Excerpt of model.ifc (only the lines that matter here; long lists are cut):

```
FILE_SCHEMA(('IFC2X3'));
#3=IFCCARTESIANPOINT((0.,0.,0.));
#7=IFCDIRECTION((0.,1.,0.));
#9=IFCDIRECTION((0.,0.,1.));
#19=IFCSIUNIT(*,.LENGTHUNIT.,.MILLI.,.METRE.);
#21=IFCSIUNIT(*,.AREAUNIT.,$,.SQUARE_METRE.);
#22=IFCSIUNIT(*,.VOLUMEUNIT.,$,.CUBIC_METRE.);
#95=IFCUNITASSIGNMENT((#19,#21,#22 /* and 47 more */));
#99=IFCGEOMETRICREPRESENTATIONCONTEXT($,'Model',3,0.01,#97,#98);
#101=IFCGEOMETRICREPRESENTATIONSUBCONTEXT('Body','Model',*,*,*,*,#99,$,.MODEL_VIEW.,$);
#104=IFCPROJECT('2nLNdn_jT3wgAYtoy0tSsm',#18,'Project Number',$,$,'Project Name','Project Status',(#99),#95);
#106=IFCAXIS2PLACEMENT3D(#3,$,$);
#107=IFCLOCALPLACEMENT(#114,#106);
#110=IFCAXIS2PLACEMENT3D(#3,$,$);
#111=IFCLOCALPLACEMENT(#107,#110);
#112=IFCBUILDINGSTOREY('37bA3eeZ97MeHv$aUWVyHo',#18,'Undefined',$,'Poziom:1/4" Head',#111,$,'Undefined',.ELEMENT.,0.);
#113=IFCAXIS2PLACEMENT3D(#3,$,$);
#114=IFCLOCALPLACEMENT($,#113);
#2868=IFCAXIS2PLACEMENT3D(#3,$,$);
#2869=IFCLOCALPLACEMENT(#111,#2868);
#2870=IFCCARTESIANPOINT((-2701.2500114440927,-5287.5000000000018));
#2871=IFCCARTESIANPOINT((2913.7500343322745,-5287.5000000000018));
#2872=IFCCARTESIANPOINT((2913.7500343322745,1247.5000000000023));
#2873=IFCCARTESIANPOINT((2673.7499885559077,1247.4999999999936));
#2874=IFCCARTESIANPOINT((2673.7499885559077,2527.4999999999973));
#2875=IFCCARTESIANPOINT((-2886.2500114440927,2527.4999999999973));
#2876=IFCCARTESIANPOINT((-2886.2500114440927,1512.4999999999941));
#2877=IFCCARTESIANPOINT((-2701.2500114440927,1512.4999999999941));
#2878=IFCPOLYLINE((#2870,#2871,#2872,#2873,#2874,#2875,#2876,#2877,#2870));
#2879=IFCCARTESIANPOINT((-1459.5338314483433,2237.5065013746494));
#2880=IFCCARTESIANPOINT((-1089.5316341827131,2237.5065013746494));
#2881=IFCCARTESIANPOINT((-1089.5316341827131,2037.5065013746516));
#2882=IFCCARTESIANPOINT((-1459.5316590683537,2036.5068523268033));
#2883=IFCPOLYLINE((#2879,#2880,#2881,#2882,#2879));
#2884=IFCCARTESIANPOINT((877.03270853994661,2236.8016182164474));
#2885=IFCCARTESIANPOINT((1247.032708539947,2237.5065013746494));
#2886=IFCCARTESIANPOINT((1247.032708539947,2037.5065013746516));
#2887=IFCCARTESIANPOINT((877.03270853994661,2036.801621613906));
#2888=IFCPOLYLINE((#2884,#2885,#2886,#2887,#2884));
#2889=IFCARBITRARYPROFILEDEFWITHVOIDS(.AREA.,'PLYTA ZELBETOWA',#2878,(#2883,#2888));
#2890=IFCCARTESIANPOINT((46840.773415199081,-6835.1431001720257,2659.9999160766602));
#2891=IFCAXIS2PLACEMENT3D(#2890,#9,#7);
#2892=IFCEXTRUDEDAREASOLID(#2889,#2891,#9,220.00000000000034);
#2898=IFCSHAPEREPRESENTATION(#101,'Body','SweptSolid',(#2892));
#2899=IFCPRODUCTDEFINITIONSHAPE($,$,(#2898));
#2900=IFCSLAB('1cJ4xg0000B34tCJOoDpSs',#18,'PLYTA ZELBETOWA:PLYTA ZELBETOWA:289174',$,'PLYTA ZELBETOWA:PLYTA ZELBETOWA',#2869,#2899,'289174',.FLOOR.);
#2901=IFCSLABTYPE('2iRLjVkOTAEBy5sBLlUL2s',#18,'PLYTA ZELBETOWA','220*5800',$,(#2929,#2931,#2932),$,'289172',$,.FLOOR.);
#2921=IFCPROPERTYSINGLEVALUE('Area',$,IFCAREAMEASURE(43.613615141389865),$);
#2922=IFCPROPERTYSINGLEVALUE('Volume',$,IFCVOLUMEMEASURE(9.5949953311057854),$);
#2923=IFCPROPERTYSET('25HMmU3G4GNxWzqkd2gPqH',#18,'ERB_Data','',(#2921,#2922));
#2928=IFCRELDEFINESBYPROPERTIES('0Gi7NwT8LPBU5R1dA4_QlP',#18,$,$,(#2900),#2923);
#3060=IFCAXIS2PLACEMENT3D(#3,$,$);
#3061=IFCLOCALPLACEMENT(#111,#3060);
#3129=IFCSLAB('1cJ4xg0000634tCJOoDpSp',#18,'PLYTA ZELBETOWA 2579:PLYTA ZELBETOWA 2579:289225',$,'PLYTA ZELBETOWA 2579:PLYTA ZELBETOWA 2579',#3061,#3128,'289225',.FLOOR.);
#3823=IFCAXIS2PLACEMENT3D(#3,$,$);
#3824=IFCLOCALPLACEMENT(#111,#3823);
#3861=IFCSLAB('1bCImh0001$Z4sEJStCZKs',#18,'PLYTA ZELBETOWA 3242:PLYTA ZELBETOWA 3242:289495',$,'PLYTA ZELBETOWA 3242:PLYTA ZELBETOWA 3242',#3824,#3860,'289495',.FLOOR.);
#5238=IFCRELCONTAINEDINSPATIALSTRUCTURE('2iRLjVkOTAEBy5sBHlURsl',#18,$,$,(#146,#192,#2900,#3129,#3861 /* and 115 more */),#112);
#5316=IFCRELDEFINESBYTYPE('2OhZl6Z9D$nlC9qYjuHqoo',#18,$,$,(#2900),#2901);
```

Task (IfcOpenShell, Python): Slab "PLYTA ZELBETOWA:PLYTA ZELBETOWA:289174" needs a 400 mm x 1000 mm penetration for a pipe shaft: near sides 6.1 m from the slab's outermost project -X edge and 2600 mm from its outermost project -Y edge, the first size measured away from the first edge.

```python
import numpy as np
import ifcopenshell
import ifcopenshell.api.feature
import ifcopenshell.api.geometry
import ifcopenshell.api.pset
import ifcopenshell.api.root
import ifcopenshell.geom
import ifcopenshell.util.element
import ifcopenshell.util.placement
import ifcopenshell.util.representation
import ifcopenshell.util.shape
import ifcopenshell.util.unit

model = ifcopenshell.open("model.ifc")
unit_scale = ifcopenshell.util.unit.calculate_unit_scale(model)
area_scale = ifcopenshell.util.unit.calculate_unit_scale(model, "AREAUNIT")
volume_scale = ifcopenshell.util.unit.calculate_unit_scale(model, "VOLUMEUNIT")
settings = ifcopenshell.geom.settings()


def volume(element):
    """Net volume in cubic metres, openings subtracted."""
    shape = ifcopenshell.geom.create_shape(settings, element)
    return ifcopenshell.util.shape.get_volume(shape.geometry)


slab = model.by_guid("1cJ4xg0000B34tCJOoDpSs")
before = volume(slab)

# Extent in the slab's own axes, in metres. The edges named are its -X and -Y sides.
slab_shape = ifcopenshell.geom.create_shape(settings, slab)
vertices = ifcopenshell.util.shape.get_vertices(slab_shape.geometry)
x_min, y_min, bottom = vertices.min(axis=0)
top = vertices[:, 2].max()

opening = ifcopenshell.api.root.create_entity(model, ifc_class="IfcOpeningElement", name="Pipe shaft opening")
context = ifcopenshell.util.representation.get_context(model, "Model", "Body", "MODEL_VIEW")
width, depth = 0.4, 1
outline = [(0.0, 0.0), (width, 0.0), (width, depth), (0.0, depth), (0.0, 0.0)]
# Overshoot both faces by 50 mm so the cut is clean.
shape = ifcopenshell.api.geometry.add_slab_representation(
    model, context=context, depth=top - bottom + 0.1, polyline=outline
)
ifcopenshell.api.geometry.assign_representation(model, product=opening, representation=shape)

matrix = ifcopenshell.util.placement.get_local_placement(slab.ObjectPlacement)
matrix[:, 3] = matrix @ np.append(np.array([x_min + 6.1, y_min + 2.6, bottom - 0.05]) / unit_scale, 1.0)
ifcopenshell.api.geometry.edit_object_placement(model, product=opening, matrix=matrix, is_si=False)
ifcopenshell.api.feature.add_feature(model, feature=opening, element=slab)

after = volume(slab)

# Update the slab's stored quantities.
pset = model.by_id(ifcopenshell.util.element.get_pset(slab, "ERB_Data", should_inherit=False)["id"])
ifcopenshell.api.pset.edit_pset(model, pset=pset, properties={
    "Area": model.create_entity("IfcAreaMeasure", after / (top - bottom) / area_scale),
    "Volume": model.create_entity("IfcVolumeMeasure", after / volume_scale),
})

print(f"slab volume {before:.3f} -> {after:.3f} m3")

model.write("model_v2.ifc")
```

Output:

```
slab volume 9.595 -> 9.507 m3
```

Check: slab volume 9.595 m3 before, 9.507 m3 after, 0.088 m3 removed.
